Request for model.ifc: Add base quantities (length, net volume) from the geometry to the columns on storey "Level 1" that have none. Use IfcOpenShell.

First a look at what the model holds.

```python
import ifcopenshell
import ifcopenshell.util.element
import ifcopenshell.util.unit

model = ifcopenshell.open("model.ifc")
print(model.schema)
for unit_type in ("LENGTHUNIT", "AREAUNIT", "VOLUMEUNIT"):
    print(unit_type, ifcopenshell.util.unit.calculate_unit_scale(model, unit_type))
storey = next(s for s in model.by_type("IfcBuildingStorey") if s.Name == "Level 1")
columns = [e for e in ifcopenshell.util.element.get_decomposition(storey) if e.is_a("IfcColumn")]
for e in sorted(columns, key=lambda e: e.id()):
    print(e.id(), e.is_a(), e.Name, list(ifcopenshell.util.element.get_psets(e, qtos_only=True)), sep=" | ")
```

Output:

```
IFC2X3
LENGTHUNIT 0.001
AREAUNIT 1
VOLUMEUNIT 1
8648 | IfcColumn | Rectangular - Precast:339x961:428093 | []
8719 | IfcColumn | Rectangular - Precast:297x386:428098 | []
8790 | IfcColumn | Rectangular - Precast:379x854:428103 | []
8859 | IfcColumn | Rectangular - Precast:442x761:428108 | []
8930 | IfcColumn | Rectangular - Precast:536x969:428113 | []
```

```python
import ifcopenshell
import ifcopenshell.api.pset
import ifcopenshell.geom
import ifcopenshell.util.element
import ifcopenshell.util.shape
import ifcopenshell.util.unit

model = ifcopenshell.open("model.ifc")
unit_scale = ifcopenshell.util.unit.calculate_unit_scale(model)
volume_scale = ifcopenshell.util.unit.calculate_unit_scale(model, "VOLUMEUNIT")
settings = ifcopenshell.geom.settings()

storey = next(s for s in model.by_type("IfcBuildingStorey") if s.Name == "Level 1")
columns = [e for e in ifcopenshell.util.element.get_decomposition(storey) if e.is_a("IfcColumn")]

for e in sorted(columns, key=lambda e: e.id()):
    if ifcopenshell.util.element.get_psets(e, qtos_only=True, should_inherit=False):
        continue
    # Geometry comes back in metres, in the element's own axes.
    shape = ifcopenshell.geom.create_shape(settings, e)
    values = {
        "Length": ifcopenshell.util.shape.get_z(shape.geometry) / unit_scale,
        "NetVolume": ifcopenshell.util.shape.get_volume(shape.geometry) / volume_scale,
    }
    qto = ifcopenshell.api.pset.add_qto(model, product=e, name="BaseQuantities")
    ifcopenshell.api.pset.edit_qto(model, qto=qto, properties=values)
    print(e.id(), {k: round(v, 3) for k, v in values.items()})

model.write("model_edited.ifc")
```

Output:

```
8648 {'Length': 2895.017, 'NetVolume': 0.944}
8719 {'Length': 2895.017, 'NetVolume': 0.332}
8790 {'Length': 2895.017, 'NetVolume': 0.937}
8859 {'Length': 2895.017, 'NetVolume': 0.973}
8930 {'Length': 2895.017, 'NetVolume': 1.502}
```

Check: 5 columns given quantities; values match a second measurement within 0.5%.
